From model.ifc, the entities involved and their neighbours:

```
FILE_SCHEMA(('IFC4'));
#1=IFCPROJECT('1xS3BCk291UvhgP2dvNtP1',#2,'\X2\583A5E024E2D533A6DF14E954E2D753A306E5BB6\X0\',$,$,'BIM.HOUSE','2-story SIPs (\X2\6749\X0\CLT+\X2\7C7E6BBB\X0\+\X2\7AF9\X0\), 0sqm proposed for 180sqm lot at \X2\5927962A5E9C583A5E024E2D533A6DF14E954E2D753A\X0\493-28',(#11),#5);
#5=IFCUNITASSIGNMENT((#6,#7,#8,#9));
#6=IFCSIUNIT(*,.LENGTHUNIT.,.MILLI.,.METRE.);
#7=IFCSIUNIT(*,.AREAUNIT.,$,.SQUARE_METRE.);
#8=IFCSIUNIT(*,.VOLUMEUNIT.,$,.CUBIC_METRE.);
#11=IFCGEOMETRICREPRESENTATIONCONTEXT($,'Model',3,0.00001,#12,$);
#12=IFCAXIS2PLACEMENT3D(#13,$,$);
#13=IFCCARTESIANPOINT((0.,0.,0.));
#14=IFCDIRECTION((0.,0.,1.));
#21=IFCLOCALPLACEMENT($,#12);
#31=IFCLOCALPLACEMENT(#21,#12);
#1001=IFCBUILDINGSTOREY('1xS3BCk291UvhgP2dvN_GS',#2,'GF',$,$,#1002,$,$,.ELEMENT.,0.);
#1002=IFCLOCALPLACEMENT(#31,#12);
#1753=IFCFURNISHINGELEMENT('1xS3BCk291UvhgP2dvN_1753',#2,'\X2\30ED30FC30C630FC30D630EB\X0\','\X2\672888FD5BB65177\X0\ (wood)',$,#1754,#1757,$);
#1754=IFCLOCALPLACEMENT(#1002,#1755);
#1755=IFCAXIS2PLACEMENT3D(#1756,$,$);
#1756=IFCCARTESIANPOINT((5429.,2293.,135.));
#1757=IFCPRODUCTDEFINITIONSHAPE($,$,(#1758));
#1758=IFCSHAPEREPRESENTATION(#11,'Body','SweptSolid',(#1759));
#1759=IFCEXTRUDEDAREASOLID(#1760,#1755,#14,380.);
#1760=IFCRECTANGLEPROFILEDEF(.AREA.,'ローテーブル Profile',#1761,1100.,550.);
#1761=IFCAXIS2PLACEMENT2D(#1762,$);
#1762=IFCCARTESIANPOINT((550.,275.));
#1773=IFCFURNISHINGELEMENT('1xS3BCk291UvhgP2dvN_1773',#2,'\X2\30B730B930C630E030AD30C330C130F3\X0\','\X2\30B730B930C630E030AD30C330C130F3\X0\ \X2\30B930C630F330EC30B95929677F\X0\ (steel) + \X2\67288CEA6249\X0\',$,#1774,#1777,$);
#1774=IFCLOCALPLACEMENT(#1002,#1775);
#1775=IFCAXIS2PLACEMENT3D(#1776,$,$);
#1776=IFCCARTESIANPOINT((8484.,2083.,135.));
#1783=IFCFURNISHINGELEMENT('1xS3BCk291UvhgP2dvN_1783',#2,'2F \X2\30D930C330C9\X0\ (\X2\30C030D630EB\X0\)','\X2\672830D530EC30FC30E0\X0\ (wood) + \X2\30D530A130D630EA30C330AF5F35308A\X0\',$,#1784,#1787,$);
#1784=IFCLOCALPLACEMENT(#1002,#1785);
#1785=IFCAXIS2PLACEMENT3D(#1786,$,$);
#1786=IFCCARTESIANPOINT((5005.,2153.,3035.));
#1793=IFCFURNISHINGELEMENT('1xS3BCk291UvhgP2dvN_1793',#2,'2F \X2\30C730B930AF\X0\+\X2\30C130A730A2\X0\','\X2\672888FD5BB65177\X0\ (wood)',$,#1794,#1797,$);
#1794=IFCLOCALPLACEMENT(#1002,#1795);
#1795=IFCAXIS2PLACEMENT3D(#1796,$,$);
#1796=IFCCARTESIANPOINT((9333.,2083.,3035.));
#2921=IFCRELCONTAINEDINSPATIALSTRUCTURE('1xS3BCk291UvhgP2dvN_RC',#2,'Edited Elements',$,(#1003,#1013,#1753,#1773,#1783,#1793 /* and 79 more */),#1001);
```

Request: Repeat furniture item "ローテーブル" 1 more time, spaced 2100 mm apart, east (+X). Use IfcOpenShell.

```python
import numpy as np
import ifcopenshell
import ifcopenshell.api.geometry
import ifcopenshell.api.root
import ifcopenshell.util.element
import ifcopenshell.util.placement

model = ifcopenshell.open("model.ifc")


def reuse_history(source, copy):
    """copy_class also copies each property set's owner history, people and application; keep the originals."""
    for rel in copy.IsDefinedBy:
        if rel.is_a("IfcRelDefinesByProperties") and (history := rel.RelatingPropertyDefinition.OwnerHistory):
            rel.RelatingPropertyDefinition.OwnerHistory = source.OwnerHistory
            ifcopenshell.util.element.remove_deep2(model, history)


source = model.by_guid("1xS3BCk291UvhgP2dvN_1753")
base = ifcopenshell.util.placement.get_local_placement(source.ObjectPlacement)
step = np.array([1.0, 0.0, 0.0]) * 2100.0

for i in range(1, 2):
    copy = ifcopenshell.api.root.copy_class(model, product=source)
    copy.Representation = ifcopenshell.util.element.copy_deep(
        model, source.Representation, exclude=["IfcGeometricRepresentationContext", "IfcRepresentationMap"]
    )
    reuse_history(source, copy)
    matrix = base.copy()
    matrix[:3, 3] += i * step
    print("added at", matrix[:3, 3].round(3) + 0.0)
    ifcopenshell.api.geometry.edit_object_placement(model, product=copy, matrix=matrix, is_si=False)

model.write("model-out.ifc")
```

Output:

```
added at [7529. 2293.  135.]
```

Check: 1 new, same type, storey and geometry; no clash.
